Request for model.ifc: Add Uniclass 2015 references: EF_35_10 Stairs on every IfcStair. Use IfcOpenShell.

First a look at what the model holds.

```python
import ifcopenshell

model = ifcopenshell.open("model.ifc")
print(model.schema)
print("classifications:", [c.Name for c in model.by_type("IfcClassification")])
for ifc_class in ("IfcDoor", "IfcRoof", "IfcStair", "IfcWall", "IfcWindow"):
    print(ifc_class, len(model.by_type(ifc_class)))
```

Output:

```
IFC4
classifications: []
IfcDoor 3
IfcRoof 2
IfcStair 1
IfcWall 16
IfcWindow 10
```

```python
import ifcopenshell
import ifcopenshell.api.classification

model = ifcopenshell.open("model.ifc")

system = ifcopenshell.api.classification.add_classification(model, classification="Uniclass 2015")

codes = {
    "IfcStair": ("EF_35_10", "Stairs"),
}
for ifc_class, (code, name) in codes.items():
    products = model.by_type(ifc_class)
    ifcopenshell.api.classification.add_reference(
        model, products=products, classification=system, identification=code, name=name
    )
    print(code, len(products))

model.write("model_v2.ifc")
```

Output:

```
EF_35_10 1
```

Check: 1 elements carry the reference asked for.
